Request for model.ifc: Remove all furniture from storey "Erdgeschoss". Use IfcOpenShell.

First a look at what the model holds.

```python
import ifcopenshell
import ifcopenshell.util.element

model = ifcopenshell.open("model.ifc")
print(model.schema)
storey = next(s for s in model.by_type("IfcBuildingStorey") if s.Name == "Erdgeschoss")
furniture = [e for e in ifcopenshell.util.element.get_decomposition(storey) if e.is_a("IfcFurnishingElement")]
seen = {}
for e in furniture:
    element_type = ifcopenshell.util.element.get_type(e)
    name = element_type.Name if element_type not in (None, e) else None
    seen[name] = seen.get(name, 0) + 1
for name, count in sorted(seen.items(), key=str):
    print(count, "x", name)
```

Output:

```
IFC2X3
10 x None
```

```python
import ifcopenshell
import ifcopenshell.api.root
import ifcopenshell.util.element

model = ifcopenshell.open("model.ifc")

storey = next(s for s in model.by_type("IfcBuildingStorey") if s.Name == "Erdgeschoss")
furniture = [e for e in ifcopenshell.util.element.get_decomposition(storey) if e.is_a("IfcFurnishingElement")]

for e in furniture:
    ifcopenshell.api.root.remove_product(model, product=e)
print(len(furniture), "removed")

model.write("model_edited.ifc")
```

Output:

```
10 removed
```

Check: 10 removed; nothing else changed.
